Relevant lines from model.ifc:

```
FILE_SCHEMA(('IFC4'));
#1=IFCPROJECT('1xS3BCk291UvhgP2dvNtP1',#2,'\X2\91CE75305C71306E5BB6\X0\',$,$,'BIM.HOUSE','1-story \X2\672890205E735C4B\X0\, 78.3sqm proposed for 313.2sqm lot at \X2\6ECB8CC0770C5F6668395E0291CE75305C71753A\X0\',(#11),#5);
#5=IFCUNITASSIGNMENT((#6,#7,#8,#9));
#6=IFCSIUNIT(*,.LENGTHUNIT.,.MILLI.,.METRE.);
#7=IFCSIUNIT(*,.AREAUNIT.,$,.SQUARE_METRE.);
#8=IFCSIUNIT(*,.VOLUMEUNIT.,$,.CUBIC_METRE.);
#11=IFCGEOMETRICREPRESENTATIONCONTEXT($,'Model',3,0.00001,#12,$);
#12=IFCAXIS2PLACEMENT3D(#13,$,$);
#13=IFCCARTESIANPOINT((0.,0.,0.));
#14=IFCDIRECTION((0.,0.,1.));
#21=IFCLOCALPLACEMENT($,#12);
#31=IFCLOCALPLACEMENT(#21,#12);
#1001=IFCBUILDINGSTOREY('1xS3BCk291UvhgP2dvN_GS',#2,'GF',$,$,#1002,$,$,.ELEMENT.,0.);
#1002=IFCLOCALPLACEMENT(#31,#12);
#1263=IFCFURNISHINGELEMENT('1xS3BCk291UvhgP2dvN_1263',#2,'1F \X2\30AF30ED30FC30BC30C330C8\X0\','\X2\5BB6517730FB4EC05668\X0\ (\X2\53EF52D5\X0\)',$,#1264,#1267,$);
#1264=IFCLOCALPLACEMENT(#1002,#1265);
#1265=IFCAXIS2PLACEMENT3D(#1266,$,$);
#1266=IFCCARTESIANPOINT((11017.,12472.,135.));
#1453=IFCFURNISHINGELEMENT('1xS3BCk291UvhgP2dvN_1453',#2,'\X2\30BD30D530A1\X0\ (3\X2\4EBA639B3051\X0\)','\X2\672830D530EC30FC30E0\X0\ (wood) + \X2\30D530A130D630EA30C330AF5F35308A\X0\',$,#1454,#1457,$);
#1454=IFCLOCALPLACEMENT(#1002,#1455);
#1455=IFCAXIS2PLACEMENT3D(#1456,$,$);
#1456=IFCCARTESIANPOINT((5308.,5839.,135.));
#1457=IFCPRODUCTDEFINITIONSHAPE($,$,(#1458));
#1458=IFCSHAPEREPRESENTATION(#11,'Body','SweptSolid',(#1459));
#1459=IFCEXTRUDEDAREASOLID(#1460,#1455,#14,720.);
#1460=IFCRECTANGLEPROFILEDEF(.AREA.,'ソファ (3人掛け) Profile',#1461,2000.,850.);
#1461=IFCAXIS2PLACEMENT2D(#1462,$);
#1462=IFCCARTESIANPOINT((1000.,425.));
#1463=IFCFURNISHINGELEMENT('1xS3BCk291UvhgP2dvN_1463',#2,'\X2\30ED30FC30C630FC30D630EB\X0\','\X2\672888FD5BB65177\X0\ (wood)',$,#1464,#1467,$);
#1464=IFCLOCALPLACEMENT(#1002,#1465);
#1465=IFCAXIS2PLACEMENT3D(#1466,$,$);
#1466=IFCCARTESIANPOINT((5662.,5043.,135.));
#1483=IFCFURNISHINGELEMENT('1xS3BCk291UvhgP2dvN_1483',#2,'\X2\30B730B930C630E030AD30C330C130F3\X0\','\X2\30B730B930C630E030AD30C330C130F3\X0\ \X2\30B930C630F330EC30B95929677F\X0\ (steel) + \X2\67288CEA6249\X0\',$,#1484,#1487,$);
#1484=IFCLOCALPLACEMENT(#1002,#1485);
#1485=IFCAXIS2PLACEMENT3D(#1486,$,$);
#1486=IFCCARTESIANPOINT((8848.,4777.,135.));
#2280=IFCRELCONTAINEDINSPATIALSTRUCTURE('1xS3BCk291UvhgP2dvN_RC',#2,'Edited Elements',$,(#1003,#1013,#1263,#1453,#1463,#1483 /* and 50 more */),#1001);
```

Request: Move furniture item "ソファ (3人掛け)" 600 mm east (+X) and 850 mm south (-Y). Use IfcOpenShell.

```python
import ifcopenshell
import ifcopenshell.api.geometry
import ifcopenshell.util.placement
import ifcopenshell.util.unit

model = ifcopenshell.open("model.ifc")
unit_scale = ifcopenshell.util.unit.calculate_unit_scale(model)

item = model.by_id(1453)
matrix = ifcopenshell.util.placement.get_local_placement(item.ObjectPlacement)
matrix[0, 3] += 0.6 / unit_scale
matrix[1, 3] -= 0.85 / unit_scale
ifcopenshell.api.geometry.edit_object_placement(model, product=item, matrix=matrix, is_si=False)

print(ifcopenshell.util.placement.get_local_placement(item.ObjectPlacement).round(3) + 0.0)

model.write("model_edited.ifc")
```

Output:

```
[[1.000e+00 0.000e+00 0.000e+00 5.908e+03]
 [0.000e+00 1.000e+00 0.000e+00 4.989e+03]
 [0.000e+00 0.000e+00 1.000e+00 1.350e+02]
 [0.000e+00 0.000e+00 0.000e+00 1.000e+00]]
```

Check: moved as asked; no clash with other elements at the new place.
